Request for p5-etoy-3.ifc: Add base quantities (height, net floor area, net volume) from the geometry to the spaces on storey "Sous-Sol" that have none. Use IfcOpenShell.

First a look at what the model holds.

```python
import ifcopenshell
import ifcopenshell.util.element
import ifcopenshell.util.unit

model = ifcopenshell.open("p5-etoy-3.ifc")
print(model.schema)
for unit_type in ("LENGTHUNIT", "AREAUNIT", "VOLUMEUNIT"):
    print(unit_type, ifcopenshell.util.unit.calculate_unit_scale(model, unit_type))
storey = next(s for s in model.by_type("IfcBuildingStorey") if s.Name == "Sous-Sol")
spaces = [e for e in ifcopenshell.util.element.get_decomposition(storey) if e.is_a("IfcSpace")]
for e in sorted(spaces, key=lambda e: e.id()):
    print(e.id(), e.is_a(), e.Name, list(ifcopenshell.util.element.get_psets(e, qtos_only=True)), sep=" | ")
```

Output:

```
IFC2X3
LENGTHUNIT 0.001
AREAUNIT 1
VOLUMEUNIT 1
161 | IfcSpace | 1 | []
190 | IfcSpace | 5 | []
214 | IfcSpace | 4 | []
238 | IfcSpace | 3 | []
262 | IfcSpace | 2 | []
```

```python
import ifcopenshell
import ifcopenshell.api.pset
import ifcopenshell.geom
import ifcopenshell.util.element
import ifcopenshell.util.shape
import ifcopenshell.util.unit

model = ifcopenshell.open("p5-etoy-3.ifc")
unit_scale = ifcopenshell.util.unit.calculate_unit_scale(model)
area_scale = ifcopenshell.util.unit.calculate_unit_scale(model, "AREAUNIT")
volume_scale = ifcopenshell.util.unit.calculate_unit_scale(model, "VOLUMEUNIT")
settings = ifcopenshell.geom.settings()

storey = next(s for s in model.by_type("IfcBuildingStorey") if s.Name == "Sous-Sol")
spaces = [e for e in ifcopenshell.util.element.get_decomposition(storey) if e.is_a("IfcSpace")]

for e in sorted(spaces, key=lambda e: e.id()):
    if ifcopenshell.util.element.get_psets(e, qtos_only=True, should_inherit=False):
        continue
    # Geometry comes back in metres, in the element's own axes.
    shape = ifcopenshell.geom.create_shape(settings, e)
    values = {
        "Height": ifcopenshell.util.shape.get_z(shape.geometry) / unit_scale,
        "NetFloorArea": ifcopenshell.util.shape.get_footprint_area(shape.geometry) / area_scale,
        "NetVolume": ifcopenshell.util.shape.get_volume(shape.geometry) / volume_scale,
    }
    qto = ifcopenshell.api.pset.add_qto(model, product=e, name="BaseQuantities")
    ifcopenshell.api.pset.edit_qto(model, qto=qto, properties=values)
    print(e.id(), {k: round(v, 3) for k, v in values.items()})

model.write("p5-etoy-3_edited.ifc")
```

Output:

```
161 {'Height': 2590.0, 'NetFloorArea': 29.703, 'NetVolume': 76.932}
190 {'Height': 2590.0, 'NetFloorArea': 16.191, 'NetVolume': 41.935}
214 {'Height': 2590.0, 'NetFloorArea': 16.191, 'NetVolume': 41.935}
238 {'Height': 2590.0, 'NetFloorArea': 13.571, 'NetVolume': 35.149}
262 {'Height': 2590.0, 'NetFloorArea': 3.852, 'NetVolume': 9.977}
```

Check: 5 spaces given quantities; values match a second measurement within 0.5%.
